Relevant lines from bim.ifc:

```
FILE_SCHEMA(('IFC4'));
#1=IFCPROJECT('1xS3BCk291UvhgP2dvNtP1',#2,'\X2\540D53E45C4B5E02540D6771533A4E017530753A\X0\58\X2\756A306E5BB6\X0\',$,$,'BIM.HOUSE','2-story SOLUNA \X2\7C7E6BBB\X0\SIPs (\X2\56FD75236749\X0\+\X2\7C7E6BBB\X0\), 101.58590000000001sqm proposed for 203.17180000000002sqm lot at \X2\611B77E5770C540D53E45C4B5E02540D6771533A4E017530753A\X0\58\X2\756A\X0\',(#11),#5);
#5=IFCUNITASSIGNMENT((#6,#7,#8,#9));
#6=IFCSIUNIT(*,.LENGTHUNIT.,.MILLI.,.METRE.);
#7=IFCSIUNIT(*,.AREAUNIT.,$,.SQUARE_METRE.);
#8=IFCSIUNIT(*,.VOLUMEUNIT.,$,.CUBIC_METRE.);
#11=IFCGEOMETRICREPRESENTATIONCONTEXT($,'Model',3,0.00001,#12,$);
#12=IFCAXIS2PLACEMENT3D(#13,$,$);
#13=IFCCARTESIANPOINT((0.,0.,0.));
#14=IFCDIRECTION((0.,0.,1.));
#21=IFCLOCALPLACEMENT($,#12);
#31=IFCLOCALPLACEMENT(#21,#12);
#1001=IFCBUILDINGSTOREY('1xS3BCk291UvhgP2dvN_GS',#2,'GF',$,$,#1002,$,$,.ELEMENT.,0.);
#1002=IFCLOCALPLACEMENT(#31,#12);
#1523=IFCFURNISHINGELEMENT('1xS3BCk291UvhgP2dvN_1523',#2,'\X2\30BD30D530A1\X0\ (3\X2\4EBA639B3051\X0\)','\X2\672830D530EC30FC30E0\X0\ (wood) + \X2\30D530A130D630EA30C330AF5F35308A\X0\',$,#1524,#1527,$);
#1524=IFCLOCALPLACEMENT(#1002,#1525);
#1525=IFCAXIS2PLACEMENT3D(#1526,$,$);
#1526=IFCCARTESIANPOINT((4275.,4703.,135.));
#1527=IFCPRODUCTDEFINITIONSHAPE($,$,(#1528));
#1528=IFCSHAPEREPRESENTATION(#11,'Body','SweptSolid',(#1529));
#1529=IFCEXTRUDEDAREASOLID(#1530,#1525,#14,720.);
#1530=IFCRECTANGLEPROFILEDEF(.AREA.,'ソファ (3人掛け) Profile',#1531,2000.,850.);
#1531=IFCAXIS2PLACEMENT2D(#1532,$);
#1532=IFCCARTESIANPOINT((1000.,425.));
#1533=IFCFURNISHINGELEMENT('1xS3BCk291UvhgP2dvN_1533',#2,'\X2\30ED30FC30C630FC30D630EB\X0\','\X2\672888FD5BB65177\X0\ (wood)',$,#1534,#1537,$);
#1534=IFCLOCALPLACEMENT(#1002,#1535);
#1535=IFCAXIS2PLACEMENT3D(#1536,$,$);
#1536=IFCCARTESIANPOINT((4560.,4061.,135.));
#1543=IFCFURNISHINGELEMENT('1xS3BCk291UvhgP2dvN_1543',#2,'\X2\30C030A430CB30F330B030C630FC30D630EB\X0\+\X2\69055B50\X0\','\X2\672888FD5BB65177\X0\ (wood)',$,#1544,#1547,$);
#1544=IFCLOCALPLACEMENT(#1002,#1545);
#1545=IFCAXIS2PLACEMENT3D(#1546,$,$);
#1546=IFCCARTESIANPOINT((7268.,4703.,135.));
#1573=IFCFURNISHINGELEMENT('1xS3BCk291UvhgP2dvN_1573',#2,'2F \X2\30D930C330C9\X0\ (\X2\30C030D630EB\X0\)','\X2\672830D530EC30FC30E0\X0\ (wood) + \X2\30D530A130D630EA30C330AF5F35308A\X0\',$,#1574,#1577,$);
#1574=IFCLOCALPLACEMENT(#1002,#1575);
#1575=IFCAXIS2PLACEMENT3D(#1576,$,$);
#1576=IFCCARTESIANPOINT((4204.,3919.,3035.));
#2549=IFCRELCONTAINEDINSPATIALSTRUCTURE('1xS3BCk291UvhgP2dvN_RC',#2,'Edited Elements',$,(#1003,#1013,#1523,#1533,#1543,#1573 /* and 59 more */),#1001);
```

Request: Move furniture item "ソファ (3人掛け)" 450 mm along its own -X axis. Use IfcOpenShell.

```python
import ifcopenshell
import ifcopenshell.api.geometry
import ifcopenshell.util.placement
import ifcopenshell.util.unit

model = ifcopenshell.open("bim.ifc")
unit_scale = ifcopenshell.util.unit.calculate_unit_scale(model)

item = model.by_guid("1xS3BCk291UvhgP2dvN_1523")
matrix = ifcopenshell.util.placement.get_local_placement(item.ObjectPlacement)
matrix[:3, 3] -= matrix[:3, 0] * 0.45 / unit_scale
ifcopenshell.api.geometry.edit_object_placement(model, product=item, matrix=matrix, is_si=False)

print(ifcopenshell.util.placement.get_local_placement(item.ObjectPlacement).round(3) + 0.0)

model.write("bim_updated.ifc")
```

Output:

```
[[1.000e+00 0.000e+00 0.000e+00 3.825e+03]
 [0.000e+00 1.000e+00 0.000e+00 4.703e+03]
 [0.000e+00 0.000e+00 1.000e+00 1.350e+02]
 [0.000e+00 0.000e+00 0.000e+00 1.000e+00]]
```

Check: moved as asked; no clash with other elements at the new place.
